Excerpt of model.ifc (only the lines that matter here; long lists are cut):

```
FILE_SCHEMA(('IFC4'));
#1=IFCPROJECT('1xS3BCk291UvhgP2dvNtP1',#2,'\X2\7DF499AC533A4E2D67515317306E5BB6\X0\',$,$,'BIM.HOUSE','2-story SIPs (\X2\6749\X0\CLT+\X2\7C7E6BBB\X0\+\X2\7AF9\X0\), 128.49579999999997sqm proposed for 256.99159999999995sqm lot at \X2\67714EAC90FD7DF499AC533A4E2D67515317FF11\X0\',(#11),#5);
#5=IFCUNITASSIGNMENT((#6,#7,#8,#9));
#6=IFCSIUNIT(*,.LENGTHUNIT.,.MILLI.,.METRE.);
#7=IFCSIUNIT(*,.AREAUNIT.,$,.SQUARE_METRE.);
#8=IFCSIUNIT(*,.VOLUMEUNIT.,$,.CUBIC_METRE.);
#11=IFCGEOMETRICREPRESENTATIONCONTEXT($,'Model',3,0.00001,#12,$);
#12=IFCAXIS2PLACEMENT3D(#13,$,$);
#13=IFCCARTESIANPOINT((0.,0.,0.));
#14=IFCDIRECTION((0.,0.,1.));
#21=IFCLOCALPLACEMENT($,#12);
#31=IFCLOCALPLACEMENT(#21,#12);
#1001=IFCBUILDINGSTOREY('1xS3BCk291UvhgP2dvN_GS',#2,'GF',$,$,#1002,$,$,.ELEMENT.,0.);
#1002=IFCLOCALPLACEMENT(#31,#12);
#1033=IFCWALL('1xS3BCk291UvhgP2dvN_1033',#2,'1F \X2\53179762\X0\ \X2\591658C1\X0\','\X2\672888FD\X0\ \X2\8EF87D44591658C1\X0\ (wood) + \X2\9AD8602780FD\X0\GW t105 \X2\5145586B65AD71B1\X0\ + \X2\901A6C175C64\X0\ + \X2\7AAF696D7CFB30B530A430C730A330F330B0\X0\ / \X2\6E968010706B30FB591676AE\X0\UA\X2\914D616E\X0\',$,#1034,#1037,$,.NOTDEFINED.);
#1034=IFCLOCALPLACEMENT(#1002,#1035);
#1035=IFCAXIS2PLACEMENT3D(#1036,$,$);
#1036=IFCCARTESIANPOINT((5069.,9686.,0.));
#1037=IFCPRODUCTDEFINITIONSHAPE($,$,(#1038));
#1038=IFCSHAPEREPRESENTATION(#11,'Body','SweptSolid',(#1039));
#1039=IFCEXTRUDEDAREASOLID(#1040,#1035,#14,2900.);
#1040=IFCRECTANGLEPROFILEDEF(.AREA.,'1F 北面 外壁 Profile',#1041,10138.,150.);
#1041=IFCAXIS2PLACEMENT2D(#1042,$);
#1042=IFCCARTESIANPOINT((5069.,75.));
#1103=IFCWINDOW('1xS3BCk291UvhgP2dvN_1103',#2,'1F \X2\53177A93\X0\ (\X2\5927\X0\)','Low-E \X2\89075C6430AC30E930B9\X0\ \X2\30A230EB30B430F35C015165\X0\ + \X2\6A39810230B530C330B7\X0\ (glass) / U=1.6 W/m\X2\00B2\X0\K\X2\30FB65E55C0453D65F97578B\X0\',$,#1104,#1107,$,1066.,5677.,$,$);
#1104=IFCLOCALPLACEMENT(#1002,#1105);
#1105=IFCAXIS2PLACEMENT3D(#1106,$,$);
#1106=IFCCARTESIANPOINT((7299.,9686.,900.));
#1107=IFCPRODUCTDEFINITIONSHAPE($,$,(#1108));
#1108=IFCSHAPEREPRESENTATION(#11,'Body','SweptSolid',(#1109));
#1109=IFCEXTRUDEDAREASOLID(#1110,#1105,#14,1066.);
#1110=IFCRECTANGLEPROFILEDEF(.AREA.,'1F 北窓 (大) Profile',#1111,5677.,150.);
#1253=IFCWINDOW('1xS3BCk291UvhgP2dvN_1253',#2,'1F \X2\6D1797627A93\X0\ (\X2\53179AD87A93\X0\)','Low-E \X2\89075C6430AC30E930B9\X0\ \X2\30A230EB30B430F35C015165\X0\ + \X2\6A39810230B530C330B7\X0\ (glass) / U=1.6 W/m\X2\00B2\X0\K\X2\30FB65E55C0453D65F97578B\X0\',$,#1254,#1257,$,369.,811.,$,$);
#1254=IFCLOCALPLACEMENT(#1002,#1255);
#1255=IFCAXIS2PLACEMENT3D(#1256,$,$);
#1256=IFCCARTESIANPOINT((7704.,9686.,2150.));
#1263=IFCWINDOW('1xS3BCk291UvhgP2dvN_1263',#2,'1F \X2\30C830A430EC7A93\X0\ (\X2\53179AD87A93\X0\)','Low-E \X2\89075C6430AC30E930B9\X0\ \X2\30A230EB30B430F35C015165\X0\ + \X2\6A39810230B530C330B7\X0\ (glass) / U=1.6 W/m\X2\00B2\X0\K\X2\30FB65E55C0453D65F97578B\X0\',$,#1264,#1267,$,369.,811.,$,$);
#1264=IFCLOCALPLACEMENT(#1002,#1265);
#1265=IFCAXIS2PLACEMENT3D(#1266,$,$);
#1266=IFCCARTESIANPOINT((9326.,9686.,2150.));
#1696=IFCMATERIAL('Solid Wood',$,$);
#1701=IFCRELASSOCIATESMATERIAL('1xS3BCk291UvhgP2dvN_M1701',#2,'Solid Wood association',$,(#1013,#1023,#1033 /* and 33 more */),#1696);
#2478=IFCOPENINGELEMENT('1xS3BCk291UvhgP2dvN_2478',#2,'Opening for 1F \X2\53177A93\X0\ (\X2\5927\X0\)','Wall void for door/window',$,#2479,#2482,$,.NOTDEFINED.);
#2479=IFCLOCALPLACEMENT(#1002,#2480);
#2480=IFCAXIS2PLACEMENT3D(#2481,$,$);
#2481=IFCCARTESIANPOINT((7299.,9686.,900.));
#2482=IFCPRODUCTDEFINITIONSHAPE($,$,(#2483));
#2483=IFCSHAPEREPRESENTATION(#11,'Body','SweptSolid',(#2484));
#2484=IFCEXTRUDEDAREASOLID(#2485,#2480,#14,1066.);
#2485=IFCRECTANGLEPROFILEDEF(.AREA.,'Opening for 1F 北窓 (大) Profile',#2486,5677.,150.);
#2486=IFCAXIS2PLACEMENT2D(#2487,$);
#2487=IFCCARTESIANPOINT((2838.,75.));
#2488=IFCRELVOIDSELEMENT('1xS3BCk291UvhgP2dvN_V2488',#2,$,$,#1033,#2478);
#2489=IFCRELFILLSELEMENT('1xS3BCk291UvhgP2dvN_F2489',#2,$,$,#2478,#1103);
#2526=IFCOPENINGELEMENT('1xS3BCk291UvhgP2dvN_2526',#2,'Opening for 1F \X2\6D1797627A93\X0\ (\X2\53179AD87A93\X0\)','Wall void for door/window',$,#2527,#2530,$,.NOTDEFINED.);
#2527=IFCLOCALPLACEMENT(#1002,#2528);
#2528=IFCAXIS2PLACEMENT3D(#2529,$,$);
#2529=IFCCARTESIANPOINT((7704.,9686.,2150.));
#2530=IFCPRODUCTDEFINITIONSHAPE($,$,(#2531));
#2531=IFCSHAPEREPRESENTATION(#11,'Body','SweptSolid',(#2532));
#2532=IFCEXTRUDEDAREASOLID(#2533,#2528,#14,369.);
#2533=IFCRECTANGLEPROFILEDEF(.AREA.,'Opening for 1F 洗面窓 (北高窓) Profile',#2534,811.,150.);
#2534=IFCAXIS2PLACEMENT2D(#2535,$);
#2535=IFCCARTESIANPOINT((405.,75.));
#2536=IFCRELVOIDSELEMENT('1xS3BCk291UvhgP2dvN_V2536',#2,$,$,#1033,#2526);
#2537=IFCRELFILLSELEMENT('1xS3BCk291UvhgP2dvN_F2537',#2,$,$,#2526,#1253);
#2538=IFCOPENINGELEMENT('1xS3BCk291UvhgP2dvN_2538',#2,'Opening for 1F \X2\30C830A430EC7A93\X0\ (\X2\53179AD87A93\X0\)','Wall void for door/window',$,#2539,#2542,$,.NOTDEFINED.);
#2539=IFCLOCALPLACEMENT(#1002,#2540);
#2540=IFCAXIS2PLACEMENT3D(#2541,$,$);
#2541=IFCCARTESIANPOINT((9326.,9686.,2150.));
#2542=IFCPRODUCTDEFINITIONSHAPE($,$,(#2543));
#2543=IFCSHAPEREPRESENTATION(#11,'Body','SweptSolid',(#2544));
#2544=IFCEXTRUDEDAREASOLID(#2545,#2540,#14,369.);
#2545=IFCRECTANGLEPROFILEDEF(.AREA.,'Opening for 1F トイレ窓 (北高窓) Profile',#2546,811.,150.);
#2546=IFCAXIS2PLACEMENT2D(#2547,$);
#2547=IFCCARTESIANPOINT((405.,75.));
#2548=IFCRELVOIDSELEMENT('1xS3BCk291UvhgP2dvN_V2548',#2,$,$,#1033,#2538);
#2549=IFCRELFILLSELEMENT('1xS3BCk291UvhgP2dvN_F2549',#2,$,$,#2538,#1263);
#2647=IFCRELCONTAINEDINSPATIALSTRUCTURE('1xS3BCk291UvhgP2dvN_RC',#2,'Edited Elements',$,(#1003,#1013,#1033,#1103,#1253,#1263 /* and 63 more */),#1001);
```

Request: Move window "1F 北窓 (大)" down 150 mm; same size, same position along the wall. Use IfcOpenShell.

```python
import numpy as np
import ifcopenshell
import ifcopenshell.api.geometry
import ifcopenshell.util.placement
import ifcopenshell.util.unit

model = ifcopenshell.open("model.ifc")
unit_scale = ifcopenshell.util.unit.calculate_unit_scale(model)

window = model.by_guid("1xS3BCk291UvhgP2dvN_1103")
opening = window.FillsVoids[0].RelatingOpeningElement
dz = -150.0

shift = np.array([0.0, 0.0, dz])
# The window is not placed relative to its opening, so move both.
for product in (opening, window):
    matrix = ifcopenshell.util.placement.get_local_placement(product.ObjectPlacement)
    matrix[:3, 3] += shift
    ifcopenshell.api.geometry.edit_object_placement(model, product=product, matrix=matrix, is_si=False)

print(f"moved by {dz * unit_scale:+.3f} m")

model.write("model_edited.ifc")
```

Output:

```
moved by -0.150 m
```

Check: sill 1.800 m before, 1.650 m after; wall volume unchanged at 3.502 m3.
